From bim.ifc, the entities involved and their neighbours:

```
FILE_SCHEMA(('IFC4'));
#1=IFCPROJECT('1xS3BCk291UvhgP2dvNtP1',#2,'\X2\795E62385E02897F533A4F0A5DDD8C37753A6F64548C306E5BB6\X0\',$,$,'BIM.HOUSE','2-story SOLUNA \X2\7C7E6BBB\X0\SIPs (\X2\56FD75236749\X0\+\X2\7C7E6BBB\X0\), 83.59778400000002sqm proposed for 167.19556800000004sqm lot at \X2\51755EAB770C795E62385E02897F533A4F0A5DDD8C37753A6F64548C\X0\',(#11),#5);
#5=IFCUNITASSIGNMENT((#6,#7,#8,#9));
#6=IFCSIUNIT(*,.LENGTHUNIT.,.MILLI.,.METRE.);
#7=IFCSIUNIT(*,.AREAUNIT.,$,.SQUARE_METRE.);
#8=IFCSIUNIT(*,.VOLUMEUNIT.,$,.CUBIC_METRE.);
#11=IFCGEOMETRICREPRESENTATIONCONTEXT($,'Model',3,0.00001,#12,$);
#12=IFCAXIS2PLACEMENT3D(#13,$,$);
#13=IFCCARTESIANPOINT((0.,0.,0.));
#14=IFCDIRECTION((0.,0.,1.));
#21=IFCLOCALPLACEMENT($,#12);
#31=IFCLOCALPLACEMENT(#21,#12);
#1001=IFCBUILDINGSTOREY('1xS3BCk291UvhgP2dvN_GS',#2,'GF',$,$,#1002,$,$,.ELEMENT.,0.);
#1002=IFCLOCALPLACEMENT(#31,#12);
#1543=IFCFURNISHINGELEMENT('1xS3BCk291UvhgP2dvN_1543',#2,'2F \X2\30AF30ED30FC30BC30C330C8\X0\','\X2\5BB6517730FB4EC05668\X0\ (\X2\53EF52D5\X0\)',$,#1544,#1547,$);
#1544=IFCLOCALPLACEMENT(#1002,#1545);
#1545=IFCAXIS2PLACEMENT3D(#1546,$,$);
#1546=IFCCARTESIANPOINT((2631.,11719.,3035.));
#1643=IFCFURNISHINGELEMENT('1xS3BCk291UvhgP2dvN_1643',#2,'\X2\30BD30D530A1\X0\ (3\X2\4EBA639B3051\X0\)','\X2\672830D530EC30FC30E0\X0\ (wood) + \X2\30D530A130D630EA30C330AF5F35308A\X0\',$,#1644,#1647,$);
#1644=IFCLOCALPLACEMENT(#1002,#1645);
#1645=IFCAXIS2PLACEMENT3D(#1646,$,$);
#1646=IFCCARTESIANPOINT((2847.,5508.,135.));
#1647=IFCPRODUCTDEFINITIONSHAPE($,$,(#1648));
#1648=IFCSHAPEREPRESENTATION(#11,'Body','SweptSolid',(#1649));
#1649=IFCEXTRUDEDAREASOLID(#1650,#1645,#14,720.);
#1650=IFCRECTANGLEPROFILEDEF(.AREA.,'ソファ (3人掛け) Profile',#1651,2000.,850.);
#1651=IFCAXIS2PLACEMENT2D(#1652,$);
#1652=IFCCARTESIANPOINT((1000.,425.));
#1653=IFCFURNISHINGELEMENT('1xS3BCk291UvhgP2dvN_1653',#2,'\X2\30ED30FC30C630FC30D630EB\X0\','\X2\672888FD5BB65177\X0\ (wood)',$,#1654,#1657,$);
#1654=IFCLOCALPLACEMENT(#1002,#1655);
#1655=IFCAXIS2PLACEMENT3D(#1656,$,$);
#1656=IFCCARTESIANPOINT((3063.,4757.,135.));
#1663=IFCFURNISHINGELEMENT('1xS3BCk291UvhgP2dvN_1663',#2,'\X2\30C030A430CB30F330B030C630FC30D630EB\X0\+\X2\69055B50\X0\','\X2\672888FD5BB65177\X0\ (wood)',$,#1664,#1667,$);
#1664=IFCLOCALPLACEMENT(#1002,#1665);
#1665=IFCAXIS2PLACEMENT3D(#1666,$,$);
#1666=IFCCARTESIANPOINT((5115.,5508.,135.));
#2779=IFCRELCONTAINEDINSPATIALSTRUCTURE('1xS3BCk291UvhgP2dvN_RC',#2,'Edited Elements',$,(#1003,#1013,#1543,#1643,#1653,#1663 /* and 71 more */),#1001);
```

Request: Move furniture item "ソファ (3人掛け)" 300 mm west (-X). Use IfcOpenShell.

```python
import ifcopenshell
import ifcopenshell.api.geometry
import ifcopenshell.util.placement

model = ifcopenshell.open("bim.ifc")

item = model.by_guid("1xS3BCk291UvhgP2dvN_1643")
matrix = ifcopenshell.util.placement.get_local_placement(item.ObjectPlacement)
matrix[0, 3] -= 300.0
ifcopenshell.api.geometry.edit_object_placement(model, product=item, matrix=matrix, is_si=False)

print(ifcopenshell.util.placement.get_local_placement(item.ObjectPlacement).round(3) + 0.0)

model.write("bim-out.ifc")
```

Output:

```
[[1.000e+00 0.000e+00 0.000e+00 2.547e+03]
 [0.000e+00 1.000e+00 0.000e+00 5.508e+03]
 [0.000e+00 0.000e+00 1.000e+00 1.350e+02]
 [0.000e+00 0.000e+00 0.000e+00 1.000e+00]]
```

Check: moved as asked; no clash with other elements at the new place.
